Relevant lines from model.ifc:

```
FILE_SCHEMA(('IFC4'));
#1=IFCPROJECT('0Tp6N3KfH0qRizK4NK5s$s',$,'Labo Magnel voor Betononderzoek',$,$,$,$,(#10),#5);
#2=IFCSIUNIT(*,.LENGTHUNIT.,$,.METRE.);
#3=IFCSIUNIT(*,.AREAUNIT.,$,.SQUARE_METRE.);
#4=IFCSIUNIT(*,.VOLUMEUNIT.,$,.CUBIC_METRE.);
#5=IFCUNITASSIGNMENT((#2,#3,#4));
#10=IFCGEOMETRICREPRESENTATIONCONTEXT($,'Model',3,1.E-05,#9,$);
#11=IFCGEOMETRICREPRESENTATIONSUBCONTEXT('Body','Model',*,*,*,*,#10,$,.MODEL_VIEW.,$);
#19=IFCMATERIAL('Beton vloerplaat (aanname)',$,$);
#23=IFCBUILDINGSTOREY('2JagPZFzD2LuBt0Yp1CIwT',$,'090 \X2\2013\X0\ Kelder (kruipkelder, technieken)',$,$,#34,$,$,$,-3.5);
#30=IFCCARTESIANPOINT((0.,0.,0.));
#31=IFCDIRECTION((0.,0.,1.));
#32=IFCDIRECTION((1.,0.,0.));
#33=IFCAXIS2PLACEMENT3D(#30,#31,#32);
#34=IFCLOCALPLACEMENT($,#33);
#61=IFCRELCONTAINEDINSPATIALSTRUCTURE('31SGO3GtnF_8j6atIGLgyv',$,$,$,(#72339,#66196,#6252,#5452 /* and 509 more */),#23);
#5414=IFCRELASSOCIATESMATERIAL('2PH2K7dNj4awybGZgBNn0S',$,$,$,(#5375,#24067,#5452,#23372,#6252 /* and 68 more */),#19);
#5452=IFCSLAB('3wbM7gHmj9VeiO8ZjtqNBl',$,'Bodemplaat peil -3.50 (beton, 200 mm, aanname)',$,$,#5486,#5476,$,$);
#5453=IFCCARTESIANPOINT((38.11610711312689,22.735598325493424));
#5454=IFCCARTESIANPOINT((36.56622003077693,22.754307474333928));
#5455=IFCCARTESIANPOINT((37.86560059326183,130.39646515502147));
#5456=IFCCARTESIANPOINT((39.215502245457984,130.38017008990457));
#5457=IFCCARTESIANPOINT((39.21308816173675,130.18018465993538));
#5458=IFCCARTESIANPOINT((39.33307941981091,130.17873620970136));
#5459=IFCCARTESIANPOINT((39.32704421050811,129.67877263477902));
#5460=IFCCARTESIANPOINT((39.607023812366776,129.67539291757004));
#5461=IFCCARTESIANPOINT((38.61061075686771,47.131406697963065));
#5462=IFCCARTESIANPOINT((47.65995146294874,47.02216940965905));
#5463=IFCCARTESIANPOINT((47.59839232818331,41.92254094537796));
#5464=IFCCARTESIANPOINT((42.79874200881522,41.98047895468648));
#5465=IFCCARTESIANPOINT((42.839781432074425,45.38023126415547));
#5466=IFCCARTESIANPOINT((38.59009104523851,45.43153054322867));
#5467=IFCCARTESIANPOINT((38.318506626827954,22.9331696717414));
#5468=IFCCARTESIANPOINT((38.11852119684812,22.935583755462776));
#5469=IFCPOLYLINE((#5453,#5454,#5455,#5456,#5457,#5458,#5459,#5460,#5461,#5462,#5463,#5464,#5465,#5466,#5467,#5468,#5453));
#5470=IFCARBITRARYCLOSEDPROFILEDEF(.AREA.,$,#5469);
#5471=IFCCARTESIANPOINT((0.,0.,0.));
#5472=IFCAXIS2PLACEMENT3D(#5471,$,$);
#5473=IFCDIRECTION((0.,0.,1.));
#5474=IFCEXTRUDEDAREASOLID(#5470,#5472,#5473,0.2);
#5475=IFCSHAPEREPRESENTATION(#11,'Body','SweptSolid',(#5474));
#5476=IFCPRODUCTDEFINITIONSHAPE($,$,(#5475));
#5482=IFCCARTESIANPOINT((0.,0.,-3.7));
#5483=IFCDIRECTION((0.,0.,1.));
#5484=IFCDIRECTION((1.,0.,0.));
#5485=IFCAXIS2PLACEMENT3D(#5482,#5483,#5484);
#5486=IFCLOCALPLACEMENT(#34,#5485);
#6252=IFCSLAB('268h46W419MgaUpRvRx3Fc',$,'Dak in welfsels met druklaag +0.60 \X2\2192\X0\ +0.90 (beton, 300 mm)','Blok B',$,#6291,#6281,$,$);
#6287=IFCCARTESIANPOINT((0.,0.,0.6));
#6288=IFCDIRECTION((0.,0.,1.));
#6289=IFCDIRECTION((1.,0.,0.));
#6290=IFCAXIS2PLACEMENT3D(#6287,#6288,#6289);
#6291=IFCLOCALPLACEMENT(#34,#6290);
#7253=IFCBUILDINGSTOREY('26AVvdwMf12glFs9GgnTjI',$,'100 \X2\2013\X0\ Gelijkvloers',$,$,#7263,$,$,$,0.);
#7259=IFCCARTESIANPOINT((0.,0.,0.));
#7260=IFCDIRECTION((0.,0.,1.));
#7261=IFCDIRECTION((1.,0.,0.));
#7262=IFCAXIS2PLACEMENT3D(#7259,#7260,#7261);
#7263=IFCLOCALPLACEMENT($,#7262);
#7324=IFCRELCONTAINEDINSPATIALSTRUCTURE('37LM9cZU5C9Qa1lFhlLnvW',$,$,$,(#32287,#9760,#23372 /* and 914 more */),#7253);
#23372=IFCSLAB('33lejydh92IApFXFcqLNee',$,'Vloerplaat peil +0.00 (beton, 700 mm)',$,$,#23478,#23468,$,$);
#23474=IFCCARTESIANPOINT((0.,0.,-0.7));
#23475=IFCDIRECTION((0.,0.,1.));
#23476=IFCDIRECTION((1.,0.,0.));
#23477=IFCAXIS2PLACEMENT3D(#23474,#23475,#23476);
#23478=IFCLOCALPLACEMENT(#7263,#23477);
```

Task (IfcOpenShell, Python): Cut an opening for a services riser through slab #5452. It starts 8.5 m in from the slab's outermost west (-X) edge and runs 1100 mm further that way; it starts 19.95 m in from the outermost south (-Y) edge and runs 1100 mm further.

```python
import numpy as np
import ifcopenshell
import ifcopenshell.api.feature
import ifcopenshell.api.geometry
import ifcopenshell.api.root
import ifcopenshell.geom
import ifcopenshell.util.placement
import ifcopenshell.util.representation
import ifcopenshell.util.shape
import ifcopenshell.util.unit

model = ifcopenshell.open("model.ifc")
unit_scale = ifcopenshell.util.unit.calculate_unit_scale(model)
settings = ifcopenshell.geom.settings()


def volume(element):
    """Net volume in cubic metres, openings subtracted."""
    shape = ifcopenshell.geom.create_shape(settings, element)
    return ifcopenshell.util.shape.get_volume(shape.geometry)


slab = model.by_guid("3wbM7gHmj9VeiO8ZjtqNBl")
before = volume(slab)

# Extent in the slab's own axes, in metres. The edges named are its -X and -Y sides.
slab_shape = ifcopenshell.geom.create_shape(settings, slab)
vertices = ifcopenshell.util.shape.get_vertices(slab_shape.geometry)
x_min, y_min, bottom = vertices.min(axis=0)
top = vertices[:, 2].max()

opening = ifcopenshell.api.root.create_entity(model, ifc_class="IfcOpeningElement", name="Services riser opening", predefined_type="OPENING")
context = ifcopenshell.util.representation.get_context(model, "Model", "Body", "MODEL_VIEW")
width, depth = 1.1, 1.1
outline = [(0.0, 0.0), (width, 0.0), (width, depth), (0.0, depth), (0.0, 0.0)]
# Overshoot both faces by 50 mm so the cut is clean.
shape = ifcopenshell.api.geometry.add_slab_representation(
    model, context=context, depth=top - bottom + 0.1, polyline=outline
)
ifcopenshell.api.geometry.assign_representation(model, product=opening, representation=shape)

matrix = ifcopenshell.util.placement.get_local_placement(slab.ObjectPlacement)
matrix[:, 3] = matrix @ np.append(np.array([x_min + 8.5, y_min + 19.95, bottom - 0.05]) / unit_scale, 1.0)
ifcopenshell.api.geometry.edit_object_placement(model, product=opening, matrix=matrix, is_si=False)
ifcopenshell.api.feature.add_feature(model, feature=opening, element=slab)

after = volume(slab)

print(f"slab volume {before:.3f} -> {after:.3f} m3")

model.write("model-out.ifc")
```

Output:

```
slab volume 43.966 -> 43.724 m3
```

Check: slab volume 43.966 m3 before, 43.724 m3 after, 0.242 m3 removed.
